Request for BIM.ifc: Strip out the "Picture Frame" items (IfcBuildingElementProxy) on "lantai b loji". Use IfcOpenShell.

First a look at what the model holds.

```python
import ifcopenshell
import ifcopenshell.util.element

model = ifcopenshell.open("BIM.ifc")
print(model.schema)
storey = next(s for s in model.by_type("IfcBuildingStorey") if s.Name == "lantai b loji")
proxies = [e for e in ifcopenshell.util.element.get_decomposition(storey) if e.is_a("IfcBuildingElementProxy")]
seen = {}
for e in proxies:
    element_type = ifcopenshell.util.element.get_type(e)
    name = element_type.Name if element_type not in (None, e) else None
    seen[name] = seen.get(name, 0) + 1
for name, count in sorted(seen.items(), key=str):
    print(count, "x", name)
```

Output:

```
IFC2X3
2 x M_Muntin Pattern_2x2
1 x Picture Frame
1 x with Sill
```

```python
import ifcopenshell
import ifcopenshell.api.root
import ifcopenshell.util.element

model = ifcopenshell.open("BIM.ifc")

storey = next(s for s in model.by_type("IfcBuildingStorey") if s.Name == "lantai b loji")
proxies = [e for e in ifcopenshell.util.element.get_decomposition(storey) if e.is_a("IfcBuildingElementProxy")]
targets = [e for e in proxies if (t := ifcopenshell.util.element.get_type(e)) not in (None, e) and t.Name == "Picture Frame"]

for e in targets:
    ifcopenshell.api.root.remove_product(model, product=e)
print(len(targets), "removed")

model.write("BIM_updated.ifc")
```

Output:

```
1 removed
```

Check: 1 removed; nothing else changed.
